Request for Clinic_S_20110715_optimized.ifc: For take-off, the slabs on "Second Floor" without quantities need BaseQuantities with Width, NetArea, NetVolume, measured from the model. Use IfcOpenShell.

First a look at what the model holds.

```python
import ifcopenshell
import ifcopenshell.util.element
import ifcopenshell.util.unit

model = ifcopenshell.open("Clinic_S_20110715_optimized.ifc")
print(model.schema)
for unit_type in ("LENGTHUNIT", "AREAUNIT", "VOLUMEUNIT"):
    print(unit_type, ifcopenshell.util.unit.calculate_unit_scale(model, unit_type))
storey = next(s for s in model.by_type("IfcBuildingStorey") if s.Name == "Second Floor")
slabs = [e for e in ifcopenshell.util.element.get_decomposition(storey) if e.is_a("IfcSlab")]
for e in sorted(slabs, key=lambda e: e.id()):
    print(e.id(), e.is_a(), e.Name, list(ifcopenshell.util.element.get_psets(e, qtos_only=True)), sep=" | ")
```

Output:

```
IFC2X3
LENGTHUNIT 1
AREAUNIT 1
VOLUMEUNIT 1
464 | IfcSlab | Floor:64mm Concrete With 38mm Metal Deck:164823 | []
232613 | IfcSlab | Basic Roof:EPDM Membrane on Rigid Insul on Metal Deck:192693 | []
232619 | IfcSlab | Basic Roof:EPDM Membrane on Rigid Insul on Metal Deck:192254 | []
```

```python
import ifcopenshell
import ifcopenshell.api.pset
import ifcopenshell.geom
import ifcopenshell.util.element
import ifcopenshell.util.shape
import ifcopenshell.util.unit

model = ifcopenshell.open("Clinic_S_20110715_optimized.ifc")
unit_scale = ifcopenshell.util.unit.calculate_unit_scale(model)
area_scale = ifcopenshell.util.unit.calculate_unit_scale(model, "AREAUNIT")
volume_scale = ifcopenshell.util.unit.calculate_unit_scale(model, "VOLUMEUNIT")
settings = ifcopenshell.geom.settings()

storey = next(s for s in model.by_type("IfcBuildingStorey") if s.Name == "Second Floor")
slabs = [e for e in ifcopenshell.util.element.get_decomposition(storey) if e.is_a("IfcSlab")]

for e in sorted(slabs, key=lambda e: e.id()):
    if ifcopenshell.util.element.get_psets(e, qtos_only=True, should_inherit=False):
        continue
    # Geometry comes back in metres, in the element's own axes.
    shape = ifcopenshell.geom.create_shape(settings, e)
    values = {
        "Width": ifcopenshell.util.shape.get_z(shape.geometry) / unit_scale,
        "NetArea": ifcopenshell.util.shape.get_footprint_area(shape.geometry) / area_scale,
        "NetVolume": ifcopenshell.util.shape.get_volume(shape.geometry) / volume_scale,
    }
    qto = ifcopenshell.api.pset.add_qto(model, product=e, name="BaseQuantities")
    ifcopenshell.api.pset.edit_qto(model, qto=qto, properties=values)
    print(e.id(), {k: round(v, 3) for k, v in values.items()})

model.write("Clinic_S_20110715_optimized_updated.ifc")
```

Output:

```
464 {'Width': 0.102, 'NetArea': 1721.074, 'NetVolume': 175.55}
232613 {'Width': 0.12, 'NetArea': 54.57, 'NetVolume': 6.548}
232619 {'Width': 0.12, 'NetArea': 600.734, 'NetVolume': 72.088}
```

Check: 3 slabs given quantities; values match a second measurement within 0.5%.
